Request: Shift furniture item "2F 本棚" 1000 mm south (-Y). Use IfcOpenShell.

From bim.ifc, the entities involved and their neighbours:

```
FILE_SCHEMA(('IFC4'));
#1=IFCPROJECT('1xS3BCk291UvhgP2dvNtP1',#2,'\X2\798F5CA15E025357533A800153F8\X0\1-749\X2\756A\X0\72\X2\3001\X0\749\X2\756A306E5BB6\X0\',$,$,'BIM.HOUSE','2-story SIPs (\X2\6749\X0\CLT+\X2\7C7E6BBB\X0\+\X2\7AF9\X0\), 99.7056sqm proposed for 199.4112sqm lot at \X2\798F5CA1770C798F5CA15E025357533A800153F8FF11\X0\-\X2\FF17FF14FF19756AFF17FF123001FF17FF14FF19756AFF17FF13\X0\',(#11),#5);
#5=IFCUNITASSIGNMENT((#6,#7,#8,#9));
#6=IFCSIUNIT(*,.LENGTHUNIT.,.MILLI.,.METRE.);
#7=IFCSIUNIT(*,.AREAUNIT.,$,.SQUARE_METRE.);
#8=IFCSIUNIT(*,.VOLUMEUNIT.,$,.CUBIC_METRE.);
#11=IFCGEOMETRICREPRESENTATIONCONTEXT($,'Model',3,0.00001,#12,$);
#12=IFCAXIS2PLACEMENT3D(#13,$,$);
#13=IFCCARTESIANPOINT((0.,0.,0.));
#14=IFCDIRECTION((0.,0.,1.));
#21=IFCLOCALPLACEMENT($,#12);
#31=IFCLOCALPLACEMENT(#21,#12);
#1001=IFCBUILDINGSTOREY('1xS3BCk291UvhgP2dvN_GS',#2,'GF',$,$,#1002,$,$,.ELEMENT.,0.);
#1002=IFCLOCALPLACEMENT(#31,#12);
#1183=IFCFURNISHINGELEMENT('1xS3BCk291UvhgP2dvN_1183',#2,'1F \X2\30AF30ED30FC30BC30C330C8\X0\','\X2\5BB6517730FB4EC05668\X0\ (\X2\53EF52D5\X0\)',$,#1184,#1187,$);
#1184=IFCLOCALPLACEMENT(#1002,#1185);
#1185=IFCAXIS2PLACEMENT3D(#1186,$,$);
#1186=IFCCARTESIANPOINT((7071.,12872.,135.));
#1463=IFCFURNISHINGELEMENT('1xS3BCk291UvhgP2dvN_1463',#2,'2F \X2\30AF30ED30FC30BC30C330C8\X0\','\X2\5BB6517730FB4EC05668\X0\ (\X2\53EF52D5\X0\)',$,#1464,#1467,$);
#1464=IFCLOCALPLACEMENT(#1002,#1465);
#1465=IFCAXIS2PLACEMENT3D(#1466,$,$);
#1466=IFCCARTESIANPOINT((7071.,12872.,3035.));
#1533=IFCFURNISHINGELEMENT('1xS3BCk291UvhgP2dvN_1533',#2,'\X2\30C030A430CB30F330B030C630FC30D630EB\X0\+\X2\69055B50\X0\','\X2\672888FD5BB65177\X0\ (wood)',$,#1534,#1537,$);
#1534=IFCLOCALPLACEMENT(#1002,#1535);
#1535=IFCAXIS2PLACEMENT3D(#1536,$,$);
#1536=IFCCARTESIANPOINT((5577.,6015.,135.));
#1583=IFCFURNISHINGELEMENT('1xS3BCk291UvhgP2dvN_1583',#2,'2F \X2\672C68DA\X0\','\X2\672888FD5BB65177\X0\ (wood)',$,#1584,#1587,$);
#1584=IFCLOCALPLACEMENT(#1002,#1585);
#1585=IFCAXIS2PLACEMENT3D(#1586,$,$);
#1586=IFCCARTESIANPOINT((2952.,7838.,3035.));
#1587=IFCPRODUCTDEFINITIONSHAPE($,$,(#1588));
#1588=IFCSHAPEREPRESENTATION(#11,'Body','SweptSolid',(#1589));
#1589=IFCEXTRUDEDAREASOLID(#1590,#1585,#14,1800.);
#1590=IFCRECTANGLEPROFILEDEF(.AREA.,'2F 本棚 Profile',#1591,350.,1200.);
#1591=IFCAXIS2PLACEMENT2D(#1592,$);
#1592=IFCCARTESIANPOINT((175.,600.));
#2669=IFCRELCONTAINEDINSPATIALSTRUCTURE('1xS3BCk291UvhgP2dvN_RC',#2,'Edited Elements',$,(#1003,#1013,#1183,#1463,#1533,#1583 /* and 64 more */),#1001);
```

```python
import ifcopenshell
import ifcopenshell.api.geometry
import ifcopenshell.util.placement
import ifcopenshell.util.unit

model = ifcopenshell.open("bim.ifc")
unit_scale = ifcopenshell.util.unit.calculate_unit_scale(model)

item = model.by_guid("1xS3BCk291UvhgP2dvN_1583")
matrix = ifcopenshell.util.placement.get_local_placement(item.ObjectPlacement)
matrix[1, 3] -= 1 / unit_scale
ifcopenshell.api.geometry.edit_object_placement(model, product=item, matrix=matrix, is_si=False)

print(ifcopenshell.util.placement.get_local_placement(item.ObjectPlacement).round(3) + 0.0)

model.write("bim_updated.ifc")
```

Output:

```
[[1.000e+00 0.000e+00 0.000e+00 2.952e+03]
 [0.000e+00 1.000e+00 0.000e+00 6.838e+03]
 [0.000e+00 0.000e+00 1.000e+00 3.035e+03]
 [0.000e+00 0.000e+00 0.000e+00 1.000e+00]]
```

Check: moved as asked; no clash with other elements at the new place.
